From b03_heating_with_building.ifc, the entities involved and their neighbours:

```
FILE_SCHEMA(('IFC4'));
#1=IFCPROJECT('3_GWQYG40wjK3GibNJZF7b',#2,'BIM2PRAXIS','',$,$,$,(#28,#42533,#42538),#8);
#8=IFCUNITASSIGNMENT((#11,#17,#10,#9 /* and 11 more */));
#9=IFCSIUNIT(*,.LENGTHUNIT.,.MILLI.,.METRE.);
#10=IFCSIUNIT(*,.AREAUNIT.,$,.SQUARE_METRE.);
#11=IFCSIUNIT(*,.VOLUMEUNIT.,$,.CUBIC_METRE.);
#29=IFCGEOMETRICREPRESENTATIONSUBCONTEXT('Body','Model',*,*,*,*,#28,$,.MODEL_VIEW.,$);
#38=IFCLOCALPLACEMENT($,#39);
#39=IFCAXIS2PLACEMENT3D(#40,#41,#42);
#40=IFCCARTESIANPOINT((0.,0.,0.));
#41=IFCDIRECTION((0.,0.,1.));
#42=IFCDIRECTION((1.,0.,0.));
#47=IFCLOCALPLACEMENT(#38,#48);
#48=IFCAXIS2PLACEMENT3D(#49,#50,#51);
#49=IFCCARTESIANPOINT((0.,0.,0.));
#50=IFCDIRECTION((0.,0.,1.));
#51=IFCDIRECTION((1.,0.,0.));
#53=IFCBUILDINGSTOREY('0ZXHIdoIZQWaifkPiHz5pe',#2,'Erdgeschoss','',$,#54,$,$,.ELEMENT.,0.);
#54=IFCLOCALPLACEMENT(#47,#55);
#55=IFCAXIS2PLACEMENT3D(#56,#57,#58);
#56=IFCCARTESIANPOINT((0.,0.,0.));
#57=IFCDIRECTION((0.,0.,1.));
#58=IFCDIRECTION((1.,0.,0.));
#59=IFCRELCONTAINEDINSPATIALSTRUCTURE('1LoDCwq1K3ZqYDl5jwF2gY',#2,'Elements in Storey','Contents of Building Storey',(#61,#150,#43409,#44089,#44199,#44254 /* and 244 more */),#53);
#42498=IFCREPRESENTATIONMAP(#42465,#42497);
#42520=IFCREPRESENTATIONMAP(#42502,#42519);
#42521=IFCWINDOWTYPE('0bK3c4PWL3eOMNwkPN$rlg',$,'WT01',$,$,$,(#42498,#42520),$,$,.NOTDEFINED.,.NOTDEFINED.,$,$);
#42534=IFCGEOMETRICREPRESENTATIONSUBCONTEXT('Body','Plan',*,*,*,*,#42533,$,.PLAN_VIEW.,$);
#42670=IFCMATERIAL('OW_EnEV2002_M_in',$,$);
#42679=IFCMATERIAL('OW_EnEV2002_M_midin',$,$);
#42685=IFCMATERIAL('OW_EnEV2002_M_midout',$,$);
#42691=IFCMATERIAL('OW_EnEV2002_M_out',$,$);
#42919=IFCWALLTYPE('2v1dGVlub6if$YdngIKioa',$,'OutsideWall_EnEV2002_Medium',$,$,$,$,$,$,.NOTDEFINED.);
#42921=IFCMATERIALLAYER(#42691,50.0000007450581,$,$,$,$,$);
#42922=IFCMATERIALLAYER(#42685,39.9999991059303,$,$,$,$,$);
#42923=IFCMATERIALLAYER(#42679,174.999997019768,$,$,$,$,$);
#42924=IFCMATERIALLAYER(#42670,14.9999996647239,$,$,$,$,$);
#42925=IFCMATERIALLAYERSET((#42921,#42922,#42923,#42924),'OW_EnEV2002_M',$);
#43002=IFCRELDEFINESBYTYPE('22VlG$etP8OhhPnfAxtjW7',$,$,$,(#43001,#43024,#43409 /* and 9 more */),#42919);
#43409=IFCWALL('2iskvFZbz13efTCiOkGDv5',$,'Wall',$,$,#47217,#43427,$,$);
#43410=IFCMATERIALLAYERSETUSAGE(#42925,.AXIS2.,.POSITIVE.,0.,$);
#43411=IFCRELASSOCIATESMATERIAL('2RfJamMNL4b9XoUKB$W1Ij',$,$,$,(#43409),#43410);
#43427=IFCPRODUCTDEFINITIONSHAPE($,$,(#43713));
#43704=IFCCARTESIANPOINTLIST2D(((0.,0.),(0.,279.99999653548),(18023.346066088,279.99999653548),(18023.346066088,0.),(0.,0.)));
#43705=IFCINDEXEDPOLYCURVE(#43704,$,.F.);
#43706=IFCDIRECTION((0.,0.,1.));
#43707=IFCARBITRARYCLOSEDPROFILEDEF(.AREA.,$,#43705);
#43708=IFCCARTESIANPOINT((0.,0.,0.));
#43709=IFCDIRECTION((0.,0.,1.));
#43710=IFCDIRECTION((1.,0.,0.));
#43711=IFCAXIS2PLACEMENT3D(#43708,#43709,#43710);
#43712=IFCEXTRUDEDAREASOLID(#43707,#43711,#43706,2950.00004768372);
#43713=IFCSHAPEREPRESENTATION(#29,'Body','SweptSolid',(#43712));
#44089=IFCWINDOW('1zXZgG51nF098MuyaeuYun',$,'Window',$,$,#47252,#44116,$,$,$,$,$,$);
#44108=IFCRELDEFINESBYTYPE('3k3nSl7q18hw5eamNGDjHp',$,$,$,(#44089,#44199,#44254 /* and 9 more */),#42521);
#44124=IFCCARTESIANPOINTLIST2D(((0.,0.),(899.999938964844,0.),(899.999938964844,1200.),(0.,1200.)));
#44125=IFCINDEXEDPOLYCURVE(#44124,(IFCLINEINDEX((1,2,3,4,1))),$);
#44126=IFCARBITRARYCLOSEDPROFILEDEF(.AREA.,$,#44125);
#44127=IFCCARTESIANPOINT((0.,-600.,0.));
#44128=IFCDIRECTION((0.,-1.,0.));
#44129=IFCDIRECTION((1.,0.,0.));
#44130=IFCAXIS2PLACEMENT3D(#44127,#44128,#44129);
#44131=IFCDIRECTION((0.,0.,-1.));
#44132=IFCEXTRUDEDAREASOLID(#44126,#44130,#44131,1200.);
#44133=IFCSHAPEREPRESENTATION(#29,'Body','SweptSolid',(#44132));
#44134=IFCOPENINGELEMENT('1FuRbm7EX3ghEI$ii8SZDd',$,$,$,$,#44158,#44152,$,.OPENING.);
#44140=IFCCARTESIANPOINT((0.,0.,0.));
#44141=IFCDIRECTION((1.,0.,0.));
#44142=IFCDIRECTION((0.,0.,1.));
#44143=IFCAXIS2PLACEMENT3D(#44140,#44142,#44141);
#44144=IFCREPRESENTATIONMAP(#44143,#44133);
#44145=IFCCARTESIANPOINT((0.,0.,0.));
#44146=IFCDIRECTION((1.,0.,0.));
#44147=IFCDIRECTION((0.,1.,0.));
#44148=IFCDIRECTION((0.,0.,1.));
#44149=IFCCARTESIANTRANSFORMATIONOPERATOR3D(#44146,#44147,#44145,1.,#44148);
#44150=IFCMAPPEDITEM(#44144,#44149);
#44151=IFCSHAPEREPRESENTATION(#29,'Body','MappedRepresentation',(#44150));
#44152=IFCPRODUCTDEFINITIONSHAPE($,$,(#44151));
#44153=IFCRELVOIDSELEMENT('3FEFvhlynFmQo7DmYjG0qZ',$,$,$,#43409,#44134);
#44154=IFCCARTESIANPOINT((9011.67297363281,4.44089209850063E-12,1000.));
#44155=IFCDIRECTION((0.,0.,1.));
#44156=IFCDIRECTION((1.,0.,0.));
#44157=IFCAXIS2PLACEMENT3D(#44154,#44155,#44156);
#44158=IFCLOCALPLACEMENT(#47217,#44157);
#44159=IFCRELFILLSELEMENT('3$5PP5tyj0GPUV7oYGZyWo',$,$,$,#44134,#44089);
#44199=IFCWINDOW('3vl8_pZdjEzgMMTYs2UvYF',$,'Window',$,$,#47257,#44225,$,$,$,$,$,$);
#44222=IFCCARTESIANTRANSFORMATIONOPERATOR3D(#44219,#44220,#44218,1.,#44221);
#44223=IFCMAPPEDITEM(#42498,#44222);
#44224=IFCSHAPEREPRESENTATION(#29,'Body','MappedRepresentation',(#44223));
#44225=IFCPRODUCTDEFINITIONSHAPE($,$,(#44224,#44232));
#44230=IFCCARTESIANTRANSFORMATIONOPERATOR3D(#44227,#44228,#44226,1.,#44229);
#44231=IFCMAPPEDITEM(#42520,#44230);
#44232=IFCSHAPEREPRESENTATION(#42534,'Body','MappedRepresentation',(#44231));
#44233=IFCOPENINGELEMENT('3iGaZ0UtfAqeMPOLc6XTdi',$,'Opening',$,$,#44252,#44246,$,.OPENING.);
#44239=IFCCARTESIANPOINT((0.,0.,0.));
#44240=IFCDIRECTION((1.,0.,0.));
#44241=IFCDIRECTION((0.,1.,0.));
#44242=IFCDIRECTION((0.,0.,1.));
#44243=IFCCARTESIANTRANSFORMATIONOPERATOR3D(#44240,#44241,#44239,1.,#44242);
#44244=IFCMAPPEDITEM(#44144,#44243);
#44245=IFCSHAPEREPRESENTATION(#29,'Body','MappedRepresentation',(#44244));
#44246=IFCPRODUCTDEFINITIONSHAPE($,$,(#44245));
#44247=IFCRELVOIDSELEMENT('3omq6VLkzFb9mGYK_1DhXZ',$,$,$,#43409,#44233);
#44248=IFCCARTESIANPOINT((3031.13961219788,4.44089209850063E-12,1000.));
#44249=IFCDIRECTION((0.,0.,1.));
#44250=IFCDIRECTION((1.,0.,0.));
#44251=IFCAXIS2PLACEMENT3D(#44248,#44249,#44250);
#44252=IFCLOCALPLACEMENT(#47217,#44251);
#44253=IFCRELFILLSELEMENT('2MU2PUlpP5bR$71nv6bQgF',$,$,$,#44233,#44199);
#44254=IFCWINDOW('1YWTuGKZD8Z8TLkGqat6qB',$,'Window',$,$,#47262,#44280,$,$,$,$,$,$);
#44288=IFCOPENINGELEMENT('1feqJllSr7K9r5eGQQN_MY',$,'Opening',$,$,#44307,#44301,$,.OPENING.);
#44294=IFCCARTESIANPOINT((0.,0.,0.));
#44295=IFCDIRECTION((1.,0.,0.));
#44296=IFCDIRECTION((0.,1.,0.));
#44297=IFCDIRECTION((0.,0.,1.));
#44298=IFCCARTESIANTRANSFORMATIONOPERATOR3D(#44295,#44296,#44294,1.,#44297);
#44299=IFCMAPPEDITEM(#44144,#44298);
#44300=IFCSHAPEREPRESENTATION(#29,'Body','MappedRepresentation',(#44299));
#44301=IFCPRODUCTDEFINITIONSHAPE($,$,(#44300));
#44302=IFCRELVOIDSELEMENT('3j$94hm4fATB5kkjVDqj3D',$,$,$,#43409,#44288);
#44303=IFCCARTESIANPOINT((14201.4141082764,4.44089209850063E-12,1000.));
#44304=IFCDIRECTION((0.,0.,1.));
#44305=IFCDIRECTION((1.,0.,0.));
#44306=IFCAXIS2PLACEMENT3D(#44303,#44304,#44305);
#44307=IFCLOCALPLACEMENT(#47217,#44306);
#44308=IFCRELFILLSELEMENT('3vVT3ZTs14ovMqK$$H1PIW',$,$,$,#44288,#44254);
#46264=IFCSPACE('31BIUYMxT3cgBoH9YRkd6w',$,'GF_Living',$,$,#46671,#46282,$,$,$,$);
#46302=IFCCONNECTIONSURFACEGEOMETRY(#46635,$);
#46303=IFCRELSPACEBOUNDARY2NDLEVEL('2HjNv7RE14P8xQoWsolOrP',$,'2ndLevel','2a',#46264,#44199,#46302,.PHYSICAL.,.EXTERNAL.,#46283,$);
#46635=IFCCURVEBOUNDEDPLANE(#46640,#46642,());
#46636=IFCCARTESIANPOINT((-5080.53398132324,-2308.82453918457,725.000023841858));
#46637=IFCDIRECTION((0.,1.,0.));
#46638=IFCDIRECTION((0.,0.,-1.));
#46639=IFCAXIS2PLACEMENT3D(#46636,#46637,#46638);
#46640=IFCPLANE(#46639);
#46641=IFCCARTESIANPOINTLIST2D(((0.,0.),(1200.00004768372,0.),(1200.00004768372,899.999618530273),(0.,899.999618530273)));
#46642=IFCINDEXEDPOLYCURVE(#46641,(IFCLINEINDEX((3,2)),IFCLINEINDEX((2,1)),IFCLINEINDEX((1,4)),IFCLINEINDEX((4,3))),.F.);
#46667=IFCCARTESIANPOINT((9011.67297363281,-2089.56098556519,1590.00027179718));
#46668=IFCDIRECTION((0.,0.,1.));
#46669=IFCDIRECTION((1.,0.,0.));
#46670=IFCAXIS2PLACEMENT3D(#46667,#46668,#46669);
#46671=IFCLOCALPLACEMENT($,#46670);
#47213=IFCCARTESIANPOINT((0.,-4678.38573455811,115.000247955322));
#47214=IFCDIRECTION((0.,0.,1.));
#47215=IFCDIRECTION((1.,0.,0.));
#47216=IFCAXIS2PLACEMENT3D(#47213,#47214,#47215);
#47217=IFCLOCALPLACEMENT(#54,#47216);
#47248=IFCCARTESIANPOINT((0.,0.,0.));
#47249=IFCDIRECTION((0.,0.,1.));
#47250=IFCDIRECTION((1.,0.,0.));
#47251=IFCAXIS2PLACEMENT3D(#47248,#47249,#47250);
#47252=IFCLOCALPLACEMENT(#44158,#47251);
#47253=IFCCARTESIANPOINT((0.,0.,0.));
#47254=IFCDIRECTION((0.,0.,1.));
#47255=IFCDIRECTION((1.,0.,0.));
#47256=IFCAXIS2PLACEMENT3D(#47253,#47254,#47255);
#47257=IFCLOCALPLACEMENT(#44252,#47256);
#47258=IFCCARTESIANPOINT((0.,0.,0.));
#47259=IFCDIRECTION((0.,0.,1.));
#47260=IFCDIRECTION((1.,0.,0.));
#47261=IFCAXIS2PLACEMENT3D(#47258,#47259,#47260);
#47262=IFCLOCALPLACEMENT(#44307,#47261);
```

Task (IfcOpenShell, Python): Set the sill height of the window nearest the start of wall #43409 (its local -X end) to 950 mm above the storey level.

```python
import numpy as np
import ifcopenshell
import ifcopenshell.api.geometry
import ifcopenshell.geom
import ifcopenshell.util.element
import ifcopenshell.util.placement
import ifcopenshell.util.shape
import ifcopenshell.util.unit

model = ifcopenshell.open("b03_heating_with_building.ifc")
unit_scale = ifcopenshell.util.unit.calculate_unit_scale(model)

window = model.by_id(44199)
opening = window.FillsVoids[0].RelatingOpeningElement
storey = ifcopenshell.util.element.get_container(window, ifc_class="IfcBuildingStorey")
level = ifcopenshell.util.placement.get_local_placement(storey.ObjectPlacement)[2, 3]

# The opening's origin need not be at the sill, so measure its lowest point.
shape = ifcopenshell.geom.create_shape(ifcopenshell.geom.settings(), opening)
bottom = ifcopenshell.util.shape.get_shape_bottom_elevation(shape, shape.geometry) / unit_scale
dz = level + 0.95 / unit_scale - bottom

shift = np.array([0.0, 0.0, dz])
# The window is placed relative to its opening, so it follows when the opening moves.
matrix = ifcopenshell.util.placement.get_local_placement(opening.ObjectPlacement)
matrix[:3, 3] += shift
ifcopenshell.api.geometry.edit_object_placement(
    model, product=opening, matrix=matrix, is_si=False, should_transform_children=True
)

# Space boundary surfaces are stored in each space's coordinates; move them too.
for rel in window.ProvidesBoundaries:
    if not rel.ConnectionGeometry:
        continue
    surface = rel.ConnectionGeometry.SurfaceOnRelatingElement.BasisSurface
    space_matrix = ifcopenshell.util.placement.get_local_placement(rel.RelatingSpace.ObjectPlacement)
    point = np.array(surface.Position.Location.Coordinates) + space_matrix[:3, :3].T @ shift
    surface.Position = model.createIfcAxis2Placement3D(
        model.createIfcCartesianPoint(point.tolist()), surface.Position.Axis, surface.Position.RefDirection
    )

print(f"moved by {dz * unit_scale:+.3f} m")

model.write("b03_heating_with_building-out.ifc")
```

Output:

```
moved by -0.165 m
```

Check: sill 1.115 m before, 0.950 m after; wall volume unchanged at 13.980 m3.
